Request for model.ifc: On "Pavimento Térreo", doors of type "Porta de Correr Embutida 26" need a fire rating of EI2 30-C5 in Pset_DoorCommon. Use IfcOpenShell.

First a look at what the model holds.

```python
import ifcopenshell
import ifcopenshell.util.element

model = ifcopenshell.open("model.ifc")
print(model.schema)
storey = next(s for s in model.by_type("IfcBuildingStorey") if s.Name == "Pavimento Térreo")
doors = [e for e in ifcopenshell.util.element.get_decomposition(storey) if e.is_a("IfcDoor")]
seen = {}
for e in doors:
    element_type = ifcopenshell.util.element.get_type(e)
    key = (element_type.Name if element_type != e and element_type else None, ifcopenshell.util.element.get_pset(e, "Pset_DoorCommon", "FireRating"))
    seen[key] = seen.get(key, 0) + 1
for (name, value), count in sorted(seen.items(), key=str):
    print(count, "x", name, "|", value)
```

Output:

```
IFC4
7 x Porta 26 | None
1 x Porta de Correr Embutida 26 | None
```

```python
import ifcopenshell
import ifcopenshell.api.pset
import ifcopenshell.util.element

model = ifcopenshell.open("model.ifc")

storey = next(s for s in model.by_type("IfcBuildingStorey") if s.Name == "Pavimento Térreo")
doors = [e for e in ifcopenshell.util.element.get_decomposition(storey) if e.is_a("IfcDoor")]

count = 0
for e in doors:
    element_type = ifcopenshell.util.element.get_type(e)
    if element_type in (None, e) or element_type.Name != "Porta de Correr Embutida 26":
        continue
    # add_pset returns the element's existing set when there is one.
    pset = ifcopenshell.api.pset.add_pset(model, product=e, name="Pset_DoorCommon")
    ifcopenshell.api.pset.edit_pset(model, pset=pset, properties={"FireRating": "EI2 30-C5"})
    count += 1

print(count, "doors updated")

model.write("model_rev.ifc")
```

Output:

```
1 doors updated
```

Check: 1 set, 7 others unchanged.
